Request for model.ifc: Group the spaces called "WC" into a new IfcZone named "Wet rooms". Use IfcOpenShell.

First a look at what the model holds.

```python
import ifcopenshell

model = ifcopenshell.open("model.ifc")
print(model.schema)
seen = {}
for space in model.by_type("IfcSpace"):
    seen[space.LongName] = seen.get(space.LongName, 0) + 1
for name, count in sorted(seen.items(), key=str):
    print(count, "x", name)
print("zones:", [z.Name for z in model.by_type("IfcZone")][:20])
```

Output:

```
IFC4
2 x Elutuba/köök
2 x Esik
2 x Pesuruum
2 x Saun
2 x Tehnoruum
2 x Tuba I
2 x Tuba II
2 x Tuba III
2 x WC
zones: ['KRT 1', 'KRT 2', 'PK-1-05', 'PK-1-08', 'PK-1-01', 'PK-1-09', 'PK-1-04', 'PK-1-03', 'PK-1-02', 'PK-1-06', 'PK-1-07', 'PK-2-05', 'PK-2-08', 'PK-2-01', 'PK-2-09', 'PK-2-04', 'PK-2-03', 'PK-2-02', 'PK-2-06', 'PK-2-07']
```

```python
import ifcopenshell
import ifcopenshell.api.group
import ifcopenshell.api.root

model = ifcopenshell.open("model.ifc")

names = {"WC"}
spaces = [s for s in model.by_type("IfcSpace") if s.LongName in names]

zone = ifcopenshell.api.root.create_entity(model, ifc_class="IfcZone", name="Wet rooms")
ifcopenshell.api.group.assign_group(model, products=spaces, group=zone)
print(len(spaces), "spaces in", zone.Name)

model.write("model_edited.ifc")
```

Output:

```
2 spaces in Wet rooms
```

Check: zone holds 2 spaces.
